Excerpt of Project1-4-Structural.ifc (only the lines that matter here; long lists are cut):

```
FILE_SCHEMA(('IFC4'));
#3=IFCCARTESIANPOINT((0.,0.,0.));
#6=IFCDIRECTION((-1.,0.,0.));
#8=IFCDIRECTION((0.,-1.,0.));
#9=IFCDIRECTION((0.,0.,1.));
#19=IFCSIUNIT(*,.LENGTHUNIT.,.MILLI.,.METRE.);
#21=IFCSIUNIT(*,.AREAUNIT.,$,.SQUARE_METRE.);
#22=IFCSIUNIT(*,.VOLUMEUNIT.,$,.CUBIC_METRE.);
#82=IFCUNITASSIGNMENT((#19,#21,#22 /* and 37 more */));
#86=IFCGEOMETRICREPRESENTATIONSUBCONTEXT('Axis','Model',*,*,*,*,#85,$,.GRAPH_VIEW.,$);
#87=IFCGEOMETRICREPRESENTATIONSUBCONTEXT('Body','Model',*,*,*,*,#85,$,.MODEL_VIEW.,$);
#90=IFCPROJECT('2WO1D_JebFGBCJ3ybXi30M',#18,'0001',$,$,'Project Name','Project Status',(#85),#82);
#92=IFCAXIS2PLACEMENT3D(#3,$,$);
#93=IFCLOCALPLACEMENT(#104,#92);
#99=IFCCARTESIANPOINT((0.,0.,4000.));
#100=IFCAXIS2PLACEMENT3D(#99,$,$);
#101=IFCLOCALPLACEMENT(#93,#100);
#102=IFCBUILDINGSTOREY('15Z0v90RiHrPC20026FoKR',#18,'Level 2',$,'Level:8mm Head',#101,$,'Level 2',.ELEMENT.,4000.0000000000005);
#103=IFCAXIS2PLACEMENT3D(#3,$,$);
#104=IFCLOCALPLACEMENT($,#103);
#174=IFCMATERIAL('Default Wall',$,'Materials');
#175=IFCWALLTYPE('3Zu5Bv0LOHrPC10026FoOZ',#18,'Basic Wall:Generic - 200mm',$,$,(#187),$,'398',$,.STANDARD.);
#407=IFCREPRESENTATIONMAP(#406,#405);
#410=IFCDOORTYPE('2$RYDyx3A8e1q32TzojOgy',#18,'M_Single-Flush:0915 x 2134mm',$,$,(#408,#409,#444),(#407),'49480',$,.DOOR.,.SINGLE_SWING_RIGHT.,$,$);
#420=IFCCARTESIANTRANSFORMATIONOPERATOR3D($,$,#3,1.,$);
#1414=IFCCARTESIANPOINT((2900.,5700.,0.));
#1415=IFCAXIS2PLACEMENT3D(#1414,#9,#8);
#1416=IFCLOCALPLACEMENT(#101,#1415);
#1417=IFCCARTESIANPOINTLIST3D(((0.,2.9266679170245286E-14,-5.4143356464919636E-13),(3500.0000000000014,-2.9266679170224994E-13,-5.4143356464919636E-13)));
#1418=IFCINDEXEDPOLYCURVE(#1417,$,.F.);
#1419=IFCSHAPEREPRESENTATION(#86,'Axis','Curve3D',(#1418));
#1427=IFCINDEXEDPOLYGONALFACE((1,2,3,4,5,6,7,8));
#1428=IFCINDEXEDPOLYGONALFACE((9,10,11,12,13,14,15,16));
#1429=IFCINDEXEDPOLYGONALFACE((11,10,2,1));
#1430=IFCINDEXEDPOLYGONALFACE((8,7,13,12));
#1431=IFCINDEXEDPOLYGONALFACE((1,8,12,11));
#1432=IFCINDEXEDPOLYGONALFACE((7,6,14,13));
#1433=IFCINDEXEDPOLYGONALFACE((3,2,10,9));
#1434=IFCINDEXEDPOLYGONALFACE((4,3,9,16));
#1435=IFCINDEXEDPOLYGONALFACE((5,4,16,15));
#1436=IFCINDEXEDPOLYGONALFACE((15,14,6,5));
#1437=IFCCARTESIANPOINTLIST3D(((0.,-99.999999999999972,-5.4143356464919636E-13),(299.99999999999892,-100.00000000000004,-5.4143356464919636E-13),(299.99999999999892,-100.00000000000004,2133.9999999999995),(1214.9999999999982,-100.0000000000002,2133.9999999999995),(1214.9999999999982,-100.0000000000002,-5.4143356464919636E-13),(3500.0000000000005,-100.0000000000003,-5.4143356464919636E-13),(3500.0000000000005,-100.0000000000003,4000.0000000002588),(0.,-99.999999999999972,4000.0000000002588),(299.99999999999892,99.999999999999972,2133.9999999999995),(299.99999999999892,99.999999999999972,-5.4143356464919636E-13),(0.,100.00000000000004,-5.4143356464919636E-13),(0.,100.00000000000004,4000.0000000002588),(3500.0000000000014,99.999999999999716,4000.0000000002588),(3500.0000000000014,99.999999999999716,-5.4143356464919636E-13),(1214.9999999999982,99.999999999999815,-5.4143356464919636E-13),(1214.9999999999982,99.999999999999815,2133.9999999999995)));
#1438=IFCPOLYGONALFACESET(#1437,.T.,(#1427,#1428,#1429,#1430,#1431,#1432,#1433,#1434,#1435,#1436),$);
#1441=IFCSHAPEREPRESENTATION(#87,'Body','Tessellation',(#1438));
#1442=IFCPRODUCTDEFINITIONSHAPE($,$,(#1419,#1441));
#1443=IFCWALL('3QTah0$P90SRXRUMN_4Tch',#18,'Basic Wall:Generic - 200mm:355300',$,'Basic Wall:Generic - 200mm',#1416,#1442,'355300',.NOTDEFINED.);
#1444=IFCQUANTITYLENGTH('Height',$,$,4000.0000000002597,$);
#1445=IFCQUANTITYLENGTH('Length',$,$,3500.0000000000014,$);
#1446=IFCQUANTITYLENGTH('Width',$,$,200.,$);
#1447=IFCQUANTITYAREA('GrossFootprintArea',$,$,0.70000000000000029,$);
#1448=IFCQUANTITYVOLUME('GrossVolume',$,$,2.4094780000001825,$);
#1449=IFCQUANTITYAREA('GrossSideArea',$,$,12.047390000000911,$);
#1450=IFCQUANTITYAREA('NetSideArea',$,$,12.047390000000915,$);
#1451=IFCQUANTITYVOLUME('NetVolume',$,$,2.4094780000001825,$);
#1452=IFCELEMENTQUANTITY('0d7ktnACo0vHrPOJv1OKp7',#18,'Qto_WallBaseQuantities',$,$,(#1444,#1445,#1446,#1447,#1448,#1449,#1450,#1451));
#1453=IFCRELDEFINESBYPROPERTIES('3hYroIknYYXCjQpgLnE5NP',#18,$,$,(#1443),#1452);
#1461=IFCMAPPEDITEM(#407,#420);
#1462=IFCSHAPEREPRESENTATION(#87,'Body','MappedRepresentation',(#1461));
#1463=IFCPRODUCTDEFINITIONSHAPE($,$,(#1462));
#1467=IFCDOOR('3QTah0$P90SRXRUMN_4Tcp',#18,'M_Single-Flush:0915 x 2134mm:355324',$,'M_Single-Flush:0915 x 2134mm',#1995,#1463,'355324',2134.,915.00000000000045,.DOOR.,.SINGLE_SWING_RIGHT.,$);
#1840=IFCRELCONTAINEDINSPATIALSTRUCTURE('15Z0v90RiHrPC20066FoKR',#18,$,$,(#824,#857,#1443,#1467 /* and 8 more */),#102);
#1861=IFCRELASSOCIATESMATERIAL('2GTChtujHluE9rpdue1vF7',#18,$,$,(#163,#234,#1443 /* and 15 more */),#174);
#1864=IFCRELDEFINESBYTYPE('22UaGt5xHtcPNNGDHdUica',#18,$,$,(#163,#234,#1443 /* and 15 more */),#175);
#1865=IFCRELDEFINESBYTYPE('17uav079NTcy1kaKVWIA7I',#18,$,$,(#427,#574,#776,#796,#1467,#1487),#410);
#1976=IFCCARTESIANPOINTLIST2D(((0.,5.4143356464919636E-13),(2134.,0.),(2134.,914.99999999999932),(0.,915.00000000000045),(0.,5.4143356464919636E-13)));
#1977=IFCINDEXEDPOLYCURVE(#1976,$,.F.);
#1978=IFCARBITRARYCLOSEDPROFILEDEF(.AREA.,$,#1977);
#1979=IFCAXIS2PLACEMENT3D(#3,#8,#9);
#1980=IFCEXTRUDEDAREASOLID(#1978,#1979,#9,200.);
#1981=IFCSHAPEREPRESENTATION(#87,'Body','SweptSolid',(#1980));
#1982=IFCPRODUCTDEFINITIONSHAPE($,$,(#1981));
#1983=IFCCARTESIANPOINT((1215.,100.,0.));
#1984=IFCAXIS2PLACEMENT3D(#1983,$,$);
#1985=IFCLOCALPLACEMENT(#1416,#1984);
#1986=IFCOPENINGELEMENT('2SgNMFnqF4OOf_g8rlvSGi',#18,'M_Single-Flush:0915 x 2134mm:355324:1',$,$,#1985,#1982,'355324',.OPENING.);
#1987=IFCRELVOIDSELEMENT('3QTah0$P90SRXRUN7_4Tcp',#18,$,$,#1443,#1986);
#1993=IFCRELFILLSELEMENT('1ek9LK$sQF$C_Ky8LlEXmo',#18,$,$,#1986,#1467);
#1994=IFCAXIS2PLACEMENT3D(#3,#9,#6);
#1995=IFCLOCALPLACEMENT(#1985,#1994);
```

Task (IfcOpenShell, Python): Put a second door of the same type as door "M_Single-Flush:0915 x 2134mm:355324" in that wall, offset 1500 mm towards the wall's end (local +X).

```python
import ifcopenshell
import ifcopenshell.api.feature
import ifcopenshell.api.geometry
import ifcopenshell.api.pset
import ifcopenshell.api.root
import ifcopenshell.geom
import ifcopenshell.util.element
import ifcopenshell.util.placement
import ifcopenshell.util.shape
import ifcopenshell.util.unit

model = ifcopenshell.open("Project1-4-Structural.ifc")
unit_scale = ifcopenshell.util.unit.calculate_unit_scale(model)
area_scale = ifcopenshell.util.unit.calculate_unit_scale(model, "AREAUNIT")
volume_scale = ifcopenshell.util.unit.calculate_unit_scale(model, "VOLUMEUNIT")
settings = ifcopenshell.geom.settings()


def volume(element):
    """Net volume in cubic metres, openings subtracted."""
    shape = ifcopenshell.geom.create_shape(settings, element)
    return ifcopenshell.util.shape.get_volume(shape.geometry)


def reuse_history(source, copy):
    """copy_class also copies each property set's owner history, people and application; keep the originals."""
    for rel in copy.IsDefinedBy:
        if rel.is_a("IfcRelDefinesByProperties") and (history := rel.RelatingPropertyDefinition.OwnerHistory):
            rel.RelatingPropertyDefinition.OwnerHistory = source.OwnerHistory
            ifcopenshell.util.element.remove_deep2(model, history)


door = model.by_guid("3QTah0$P90SRXRUMN_4Tcp")
opening = door.FillsVoids[0].RelatingOpeningElement
wall = opening.VoidsElements[0].RelatingBuildingElement
before = volume(wall)
shift = ifcopenshell.util.placement.get_local_placement(wall.ObjectPlacement)[:3, 0] * 1.5 / unit_scale

# copy_class copies the void relationship, type, container and properties, but no geometry.
new_opening = ifcopenshell.api.root.copy_class(model, product=opening)
new_opening.Representation = ifcopenshell.util.element.copy_deep(
    model, opening.Representation, exclude=["IfcGeometricRepresentationContext", "IfcRepresentationMap"]
)
new_opening.Name = "M_Single-Flush:0915 x 2134mm"
new_opening.Tag = None
reuse_history(opening, new_opening)
new_door = ifcopenshell.api.root.copy_class(model, product=door)
new_door.Representation = ifcopenshell.util.element.copy_deep(
    model, door.Representation, exclude=["IfcGeometricRepresentationContext", "IfcRepresentationMap"]
)
new_door.Name = "M_Single-Flush:0915 x 2134mm"
new_door.Tag = None
reuse_history(door, new_door)
ifcopenshell.api.feature.add_filling(model, opening=new_opening, element=new_door)

for old, new in ((opening, new_opening), (door, new_door)):
    matrix = ifcopenshell.util.placement.get_local_placement(old.ObjectPlacement)
    matrix[:3, 3] += shift
    ifcopenshell.api.geometry.edit_object_placement(model, product=new, matrix=matrix, is_si=False)

after = volume(wall)
thickness = 0.2  # wall thickness in metres

# Update the wall's stored quantities.
qto = model.by_id(ifcopenshell.util.element.get_pset(wall, "Qto_WallBaseQuantities", should_inherit=False)["id"])
ifcopenshell.api.pset.edit_qto(model, qto=qto, properties={
    "NetSideArea": after / thickness / area_scale,
    "NetVolume": after / volume_scale,
})

print(f"wall volume {before:.3f} -> {after:.3f} m3")

model.write("Project1-4-Structural_v2.ifc")
```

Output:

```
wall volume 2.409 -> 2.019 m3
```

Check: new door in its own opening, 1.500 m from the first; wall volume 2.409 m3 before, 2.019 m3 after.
